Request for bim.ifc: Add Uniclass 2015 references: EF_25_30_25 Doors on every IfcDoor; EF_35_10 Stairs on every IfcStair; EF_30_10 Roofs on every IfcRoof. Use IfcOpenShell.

First a look at what the model holds.

```python
import ifcopenshell

model = ifcopenshell.open("bim.ifc")
print(model.schema)
print("classifications:", [c.Name for c in model.by_type("IfcClassification")])
for ifc_class in ("IfcDoor", "IfcRoof", "IfcStair", "IfcWall", "IfcWindow"):
    print(ifc_class, len(model.by_type(ifc_class)))
```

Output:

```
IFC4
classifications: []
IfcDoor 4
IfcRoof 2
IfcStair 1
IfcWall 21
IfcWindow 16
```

```python
import ifcopenshell
import ifcopenshell.api.classification

model = ifcopenshell.open("bim.ifc")

system = ifcopenshell.api.classification.add_classification(model, classification="Uniclass 2015")

codes = {
    "IfcDoor": ("EF_25_30_25", "Doors"),
    "IfcStair": ("EF_35_10", "Stairs"),
    "IfcRoof": ("EF_30_10", "Roofs"),
}
for ifc_class, (code, name) in codes.items():
    products = model.by_type(ifc_class)
    ifcopenshell.api.classification.add_reference(
        model, products=products, classification=system, identification=code, name=name
    )
    print(code, len(products))

model.write("bim_rev.ifc")
```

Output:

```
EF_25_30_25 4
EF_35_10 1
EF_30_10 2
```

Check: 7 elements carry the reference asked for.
